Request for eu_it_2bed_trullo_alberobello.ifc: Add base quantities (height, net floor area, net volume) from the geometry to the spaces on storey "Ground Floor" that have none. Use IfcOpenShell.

First a look at what the model holds.

```python
import ifcopenshell
import ifcopenshell.util.element
import ifcopenshell.util.unit

model = ifcopenshell.open("eu_it_2bed_trullo_alberobello.ifc")
print(model.schema)
for unit_type in ("LENGTHUNIT", "AREAUNIT", "VOLUMEUNIT"):
    print(unit_type, ifcopenshell.util.unit.calculate_unit_scale(model, unit_type))
storey = next(s for s in model.by_type("IfcBuildingStorey") if s.Name == "Ground Floor")
spaces = [e for e in ifcopenshell.util.element.get_decomposition(storey) if e.is_a("IfcSpace")]
for e in sorted(spaces, key=lambda e: e.id()):
    print(e.id(), e.is_a(), e.Name, list(ifcopenshell.util.element.get_psets(e, qtos_only=True)), sep=" | ")
```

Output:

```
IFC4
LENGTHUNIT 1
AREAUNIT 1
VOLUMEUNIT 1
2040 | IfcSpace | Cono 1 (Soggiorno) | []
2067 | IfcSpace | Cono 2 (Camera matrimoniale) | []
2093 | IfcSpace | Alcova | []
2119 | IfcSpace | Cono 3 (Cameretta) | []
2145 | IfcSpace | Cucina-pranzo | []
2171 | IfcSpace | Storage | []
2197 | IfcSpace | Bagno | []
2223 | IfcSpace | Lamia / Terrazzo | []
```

```python
import ifcopenshell
import ifcopenshell.api.pset
import ifcopenshell.geom
import ifcopenshell.util.element
import ifcopenshell.util.shape
import ifcopenshell.util.unit

model = ifcopenshell.open("eu_it_2bed_trullo_alberobello.ifc")
unit_scale = ifcopenshell.util.unit.calculate_unit_scale(model)
area_scale = ifcopenshell.util.unit.calculate_unit_scale(model, "AREAUNIT")
volume_scale = ifcopenshell.util.unit.calculate_unit_scale(model, "VOLUMEUNIT")
settings = ifcopenshell.geom.settings()

storey = next(s for s in model.by_type("IfcBuildingStorey") if s.Name == "Ground Floor")
spaces = [e for e in ifcopenshell.util.element.get_decomposition(storey) if e.is_a("IfcSpace")]

for e in sorted(spaces, key=lambda e: e.id()):
    if ifcopenshell.util.element.get_psets(e, qtos_only=True, should_inherit=False):
        continue
    # Geometry comes back in metres, in the element's own axes.
    shape = ifcopenshell.geom.create_shape(settings, e)
    values = {
        "Height": ifcopenshell.util.shape.get_z(shape.geometry) / unit_scale,
        "NetFloorArea": ifcopenshell.util.shape.get_footprint_area(shape.geometry) / area_scale,
        "NetVolume": ifcopenshell.util.shape.get_volume(shape.geometry) / volume_scale,
    }
    qto = ifcopenshell.api.pset.add_qto(model, product=e, name="Qto_SpaceBaseQuantities")
    ifcopenshell.api.pset.edit_qto(model, qto=qto, properties=values)
    print(e.id(), {k: round(v, 3) for k, v in values.items()})

model.write("eu_it_2bed_trullo_alberobello-out.ifc")
```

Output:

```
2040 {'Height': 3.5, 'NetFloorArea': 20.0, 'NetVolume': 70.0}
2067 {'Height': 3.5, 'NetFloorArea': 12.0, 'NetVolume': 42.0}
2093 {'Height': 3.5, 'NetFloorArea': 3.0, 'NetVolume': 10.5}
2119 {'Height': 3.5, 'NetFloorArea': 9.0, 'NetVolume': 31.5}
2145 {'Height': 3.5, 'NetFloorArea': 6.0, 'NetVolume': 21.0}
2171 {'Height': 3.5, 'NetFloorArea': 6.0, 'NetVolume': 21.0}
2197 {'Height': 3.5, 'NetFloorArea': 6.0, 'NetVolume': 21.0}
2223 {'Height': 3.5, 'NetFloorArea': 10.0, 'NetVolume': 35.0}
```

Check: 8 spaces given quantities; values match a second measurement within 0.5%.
